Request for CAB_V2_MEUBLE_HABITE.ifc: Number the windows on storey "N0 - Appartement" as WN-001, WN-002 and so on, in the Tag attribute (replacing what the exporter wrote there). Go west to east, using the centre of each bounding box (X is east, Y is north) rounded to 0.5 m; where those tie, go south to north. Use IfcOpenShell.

First a look at what the model holds.

```python
import ifcopenshell
import ifcopenshell.util.element
import ifcopenshell.util.placement

model = ifcopenshell.open("CAB_V2_MEUBLE_HABITE.ifc")
print(model.schema)
storey = next(s for s in model.by_type("IfcBuildingStorey") if s.Name == "N0 - Appartement")
windows = [e for e in ifcopenshell.util.element.get_decomposition(storey) if e.is_a("IfcWindow")]
for e in sorted(windows, key=lambda e: e.id()):
    origin = ifcopenshell.util.placement.get_local_placement(e.ObjectPlacement)[:3, 3]
    print(e.id(), e.Tag, e.Name, origin.round(2) + 0.0, sep=" | ")
```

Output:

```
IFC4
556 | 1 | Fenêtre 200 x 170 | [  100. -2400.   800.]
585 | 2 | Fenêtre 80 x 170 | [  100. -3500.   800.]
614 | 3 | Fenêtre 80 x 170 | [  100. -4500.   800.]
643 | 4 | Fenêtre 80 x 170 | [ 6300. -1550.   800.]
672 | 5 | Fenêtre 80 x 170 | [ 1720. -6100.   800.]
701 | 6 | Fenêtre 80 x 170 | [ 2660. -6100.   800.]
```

```python
import ifcopenshell
import ifcopenshell.geom
import ifcopenshell.util.element
import ifcopenshell.util.shape

model = ifcopenshell.open("CAB_V2_MEUBLE_HABITE.ifc")
settings = ifcopenshell.geom.settings()
settings.set("use-world-coords", True)


def centre(element):
    shape = ifcopenshell.geom.create_shape(settings, element)
    return ifcopenshell.util.shape.get_bbox_centroid(shape.geometry)


storey = next(s for s in model.by_type("IfcBuildingStorey") if s.Name == "N0 - Appartement")
windows = [e for e in ifcopenshell.util.element.get_decomposition(storey) if e.is_a("IfcWindow")]

# Insertion points can sit at a corner or the storey origin, so sort by the geometry (in metres).
centres = {e: centre(e) for e in windows}
windows.sort(key=lambda e: (round(centres[e][0] / 0.5), centres[e][1]))

for i, e in enumerate(windows, start=1):
    number = f"WN-0{i:02d}"
    e.Tag = number
    print(e.id(), number)

model.write("CAB_V2_MEUBLE_HABITE-out.ifc")
```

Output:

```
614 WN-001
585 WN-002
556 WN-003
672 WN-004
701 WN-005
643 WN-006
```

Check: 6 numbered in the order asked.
